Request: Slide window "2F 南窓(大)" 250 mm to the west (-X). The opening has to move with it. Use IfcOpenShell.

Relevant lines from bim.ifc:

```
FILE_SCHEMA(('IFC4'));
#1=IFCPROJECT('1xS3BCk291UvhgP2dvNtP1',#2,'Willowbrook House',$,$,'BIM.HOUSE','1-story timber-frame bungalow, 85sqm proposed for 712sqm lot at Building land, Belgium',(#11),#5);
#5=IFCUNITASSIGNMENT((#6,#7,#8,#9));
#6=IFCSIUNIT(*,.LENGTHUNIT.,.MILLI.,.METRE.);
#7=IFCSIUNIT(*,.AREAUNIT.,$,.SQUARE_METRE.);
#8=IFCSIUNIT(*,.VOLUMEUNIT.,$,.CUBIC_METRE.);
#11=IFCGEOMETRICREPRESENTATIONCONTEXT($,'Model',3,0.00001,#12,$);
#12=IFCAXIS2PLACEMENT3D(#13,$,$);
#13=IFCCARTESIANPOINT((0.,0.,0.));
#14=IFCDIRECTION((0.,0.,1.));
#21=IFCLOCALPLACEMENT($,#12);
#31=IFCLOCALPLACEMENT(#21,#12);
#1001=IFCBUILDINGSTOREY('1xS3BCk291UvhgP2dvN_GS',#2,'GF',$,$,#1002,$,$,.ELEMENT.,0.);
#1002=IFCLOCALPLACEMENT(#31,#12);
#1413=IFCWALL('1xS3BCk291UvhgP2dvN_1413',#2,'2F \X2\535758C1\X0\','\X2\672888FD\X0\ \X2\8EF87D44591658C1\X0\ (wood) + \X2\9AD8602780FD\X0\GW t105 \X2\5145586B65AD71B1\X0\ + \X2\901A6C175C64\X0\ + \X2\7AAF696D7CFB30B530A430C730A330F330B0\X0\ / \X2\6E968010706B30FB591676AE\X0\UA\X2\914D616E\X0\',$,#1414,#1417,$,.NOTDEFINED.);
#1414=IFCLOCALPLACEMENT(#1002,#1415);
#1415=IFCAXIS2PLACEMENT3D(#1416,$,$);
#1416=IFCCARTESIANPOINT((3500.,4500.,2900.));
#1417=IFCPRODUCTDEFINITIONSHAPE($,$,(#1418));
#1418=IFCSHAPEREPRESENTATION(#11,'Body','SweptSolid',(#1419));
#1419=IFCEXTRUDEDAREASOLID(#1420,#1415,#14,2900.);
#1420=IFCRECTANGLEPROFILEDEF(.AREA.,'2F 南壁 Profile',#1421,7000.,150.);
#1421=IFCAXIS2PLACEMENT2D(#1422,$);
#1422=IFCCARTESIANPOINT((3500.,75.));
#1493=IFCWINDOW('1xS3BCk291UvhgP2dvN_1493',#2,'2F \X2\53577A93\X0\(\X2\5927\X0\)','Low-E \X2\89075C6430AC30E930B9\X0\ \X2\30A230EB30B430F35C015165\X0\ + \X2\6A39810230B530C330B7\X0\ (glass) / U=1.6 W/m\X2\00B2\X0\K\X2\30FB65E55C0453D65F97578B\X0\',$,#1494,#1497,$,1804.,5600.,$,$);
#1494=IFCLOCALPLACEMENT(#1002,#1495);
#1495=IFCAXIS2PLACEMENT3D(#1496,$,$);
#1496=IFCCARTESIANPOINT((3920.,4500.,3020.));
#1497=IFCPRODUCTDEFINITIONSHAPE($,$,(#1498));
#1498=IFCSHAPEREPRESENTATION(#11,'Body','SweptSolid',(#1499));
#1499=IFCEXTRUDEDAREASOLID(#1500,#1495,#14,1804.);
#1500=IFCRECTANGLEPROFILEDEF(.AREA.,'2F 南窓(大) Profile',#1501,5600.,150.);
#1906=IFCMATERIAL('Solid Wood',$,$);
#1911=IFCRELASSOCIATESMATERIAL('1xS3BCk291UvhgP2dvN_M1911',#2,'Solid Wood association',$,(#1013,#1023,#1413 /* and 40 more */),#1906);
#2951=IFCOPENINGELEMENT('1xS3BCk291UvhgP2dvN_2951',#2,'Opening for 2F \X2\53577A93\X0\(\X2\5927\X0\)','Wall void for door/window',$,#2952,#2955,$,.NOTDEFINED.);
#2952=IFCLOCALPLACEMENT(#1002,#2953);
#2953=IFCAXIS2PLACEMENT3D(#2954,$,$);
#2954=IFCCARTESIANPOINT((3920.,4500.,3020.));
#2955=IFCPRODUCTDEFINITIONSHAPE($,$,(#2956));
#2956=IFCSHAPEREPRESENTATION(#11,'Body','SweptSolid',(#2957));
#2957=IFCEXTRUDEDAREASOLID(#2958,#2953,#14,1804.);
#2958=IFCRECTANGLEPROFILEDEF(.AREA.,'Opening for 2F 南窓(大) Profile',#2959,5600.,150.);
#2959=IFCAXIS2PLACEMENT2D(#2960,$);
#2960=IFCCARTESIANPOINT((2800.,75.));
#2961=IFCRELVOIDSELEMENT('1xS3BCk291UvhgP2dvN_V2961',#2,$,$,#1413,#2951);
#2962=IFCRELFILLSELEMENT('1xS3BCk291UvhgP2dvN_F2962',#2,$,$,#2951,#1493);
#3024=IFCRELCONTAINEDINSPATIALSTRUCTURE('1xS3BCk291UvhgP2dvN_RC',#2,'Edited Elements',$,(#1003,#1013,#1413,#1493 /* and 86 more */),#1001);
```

```python
import ifcopenshell
import ifcopenshell.api.geometry
import ifcopenshell.util.placement

model = ifcopenshell.open("bim.ifc")

window = model.by_guid("1xS3BCk291UvhgP2dvN_1493")
opening = window.FillsVoids[0].RelatingOpeningElement
wall = opening.VoidsElements[0].RelatingBuildingElement

wall_matrix = ifcopenshell.util.placement.get_local_placement(wall.ObjectPlacement)
shift = wall_matrix[:3, 0] * -250.0
before = ifcopenshell.util.placement.get_local_placement(window.ObjectPlacement)[:3, 3].copy()

# The window is not placed relative to its opening, so move both.
for product in (opening, window):
    matrix = ifcopenshell.util.placement.get_local_placement(product.ObjectPlacement)
    matrix[:3, 3] += shift
    ifcopenshell.api.geometry.edit_object_placement(model, product=product, matrix=matrix, is_si=False)

after = ifcopenshell.util.placement.get_local_placement(window.ObjectPlacement)[:3, 3]
print("window moved by", (after - before).round(3) + 0.0)

model.write("bim_updated.ifc")
```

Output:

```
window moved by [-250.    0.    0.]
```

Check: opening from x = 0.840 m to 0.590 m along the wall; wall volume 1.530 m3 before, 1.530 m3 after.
